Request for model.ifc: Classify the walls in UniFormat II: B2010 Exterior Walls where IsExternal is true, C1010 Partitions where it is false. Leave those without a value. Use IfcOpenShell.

First a look at what the model holds.

```python
import ifcopenshell
import ifcopenshell.util.element

model = ifcopenshell.open("model.ifc")
print(model.schema)
print("classifications:", [c.Name for c in model.by_type("IfcClassification")])
values = [ifcopenshell.util.element.get_pset(e, "Pset_WallCommon", "IsExternal") for e in model.by_type("IfcWall")]
for value in (True, False, None):
    print("IsExternal", value, values.count(value))
```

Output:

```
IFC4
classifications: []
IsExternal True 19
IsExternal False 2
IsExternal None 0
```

```python
import ifcopenshell
import ifcopenshell.api.classification
import ifcopenshell.util.element

model = ifcopenshell.open("model.ifc")

system = ifcopenshell.api.classification.add_classification(model, classification="UniFormat II")

walls = model.by_type("IfcWall")
external = {e: ifcopenshell.util.element.get_pset(e, "Pset_WallCommon", "IsExternal") for e in walls}
for flag, code, name in ((True, "B2010", "Exterior Walls"), (False, "C1010", "Partitions")):
    products = [e for e in walls if external[e] is flag]
    ifcopenshell.api.classification.add_reference(
        model, products=products, classification=system, identification=code, name=name
    )
    print(code, len(products))

model.write("model-out.ifc")
```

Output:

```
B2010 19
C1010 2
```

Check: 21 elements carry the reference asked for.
